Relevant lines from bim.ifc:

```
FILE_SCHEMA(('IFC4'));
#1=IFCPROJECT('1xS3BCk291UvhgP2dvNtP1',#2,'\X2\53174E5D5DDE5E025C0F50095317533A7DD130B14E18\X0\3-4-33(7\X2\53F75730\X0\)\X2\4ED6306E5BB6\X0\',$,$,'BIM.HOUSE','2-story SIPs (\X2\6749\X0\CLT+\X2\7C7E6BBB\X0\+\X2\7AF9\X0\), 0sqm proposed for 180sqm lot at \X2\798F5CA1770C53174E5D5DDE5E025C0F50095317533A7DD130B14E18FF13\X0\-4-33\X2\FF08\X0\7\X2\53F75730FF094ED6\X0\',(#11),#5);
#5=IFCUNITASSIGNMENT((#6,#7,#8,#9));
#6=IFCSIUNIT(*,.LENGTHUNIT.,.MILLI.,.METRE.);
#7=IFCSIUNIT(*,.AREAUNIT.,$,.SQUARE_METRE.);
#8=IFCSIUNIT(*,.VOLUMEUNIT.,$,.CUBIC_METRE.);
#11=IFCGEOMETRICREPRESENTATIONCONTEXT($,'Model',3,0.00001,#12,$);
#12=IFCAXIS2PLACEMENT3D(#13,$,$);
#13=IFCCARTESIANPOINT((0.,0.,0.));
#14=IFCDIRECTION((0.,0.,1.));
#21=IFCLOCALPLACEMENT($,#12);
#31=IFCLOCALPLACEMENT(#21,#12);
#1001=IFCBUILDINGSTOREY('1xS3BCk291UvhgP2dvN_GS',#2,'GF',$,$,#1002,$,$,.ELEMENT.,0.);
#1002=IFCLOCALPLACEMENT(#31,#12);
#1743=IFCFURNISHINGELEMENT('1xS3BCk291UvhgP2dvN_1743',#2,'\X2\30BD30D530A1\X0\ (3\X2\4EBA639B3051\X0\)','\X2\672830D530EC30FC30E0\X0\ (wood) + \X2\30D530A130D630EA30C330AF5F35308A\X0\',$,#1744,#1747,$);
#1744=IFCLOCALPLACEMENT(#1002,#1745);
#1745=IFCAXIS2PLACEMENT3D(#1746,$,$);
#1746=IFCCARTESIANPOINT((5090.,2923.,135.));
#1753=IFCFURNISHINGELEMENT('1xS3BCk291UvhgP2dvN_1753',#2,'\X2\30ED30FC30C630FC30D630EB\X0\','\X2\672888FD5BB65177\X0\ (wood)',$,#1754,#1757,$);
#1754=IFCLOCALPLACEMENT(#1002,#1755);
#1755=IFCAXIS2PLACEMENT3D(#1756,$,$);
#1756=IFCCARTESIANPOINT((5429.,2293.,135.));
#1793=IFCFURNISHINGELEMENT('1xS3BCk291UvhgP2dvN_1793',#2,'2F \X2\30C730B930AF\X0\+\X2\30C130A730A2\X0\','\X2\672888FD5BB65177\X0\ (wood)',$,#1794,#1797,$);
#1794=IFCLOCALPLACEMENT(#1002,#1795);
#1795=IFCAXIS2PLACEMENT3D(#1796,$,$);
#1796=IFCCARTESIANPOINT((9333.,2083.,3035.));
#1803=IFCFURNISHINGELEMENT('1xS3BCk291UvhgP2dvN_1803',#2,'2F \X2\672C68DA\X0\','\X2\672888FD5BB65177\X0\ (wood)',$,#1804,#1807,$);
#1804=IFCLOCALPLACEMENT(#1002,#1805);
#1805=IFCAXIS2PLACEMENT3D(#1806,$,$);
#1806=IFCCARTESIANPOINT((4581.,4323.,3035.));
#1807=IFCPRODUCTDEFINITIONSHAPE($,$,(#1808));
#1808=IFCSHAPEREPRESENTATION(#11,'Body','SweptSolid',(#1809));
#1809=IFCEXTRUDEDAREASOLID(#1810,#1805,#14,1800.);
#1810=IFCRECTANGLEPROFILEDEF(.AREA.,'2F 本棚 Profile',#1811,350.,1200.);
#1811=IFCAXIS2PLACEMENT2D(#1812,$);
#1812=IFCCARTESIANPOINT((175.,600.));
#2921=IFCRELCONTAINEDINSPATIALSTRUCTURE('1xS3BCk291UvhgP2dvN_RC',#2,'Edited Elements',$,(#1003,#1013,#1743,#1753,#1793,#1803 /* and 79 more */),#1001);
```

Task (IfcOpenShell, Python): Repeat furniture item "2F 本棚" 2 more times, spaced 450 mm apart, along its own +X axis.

```python
import ifcopenshell
import ifcopenshell.api.geometry
import ifcopenshell.api.root
import ifcopenshell.util.element
import ifcopenshell.util.placement

model = ifcopenshell.open("bim.ifc")


def reuse_history(source, copy):
    """copy_class also copies each property set's owner history, people and application; keep the originals."""
    for rel in copy.IsDefinedBy:
        if rel.is_a("IfcRelDefinesByProperties") and (history := rel.RelatingPropertyDefinition.OwnerHistory):
            rel.RelatingPropertyDefinition.OwnerHistory = source.OwnerHistory
            ifcopenshell.util.element.remove_deep2(model, history)


source = model.by_id(1803)
base = ifcopenshell.util.placement.get_local_placement(source.ObjectPlacement)
step = base[:3, 0] * 450.0

for i in range(1, 3):
    copy = ifcopenshell.api.root.copy_class(model, product=source)
    copy.Representation = ifcopenshell.util.element.copy_deep(
        model, source.Representation, exclude=["IfcGeometricRepresentationContext", "IfcRepresentationMap"]
    )
    reuse_history(source, copy)
    matrix = base.copy()
    matrix[:3, 3] += i * step
    print("added at", matrix[:3, 3].round(3) + 0.0)
    ifcopenshell.api.geometry.edit_object_placement(model, product=copy, matrix=matrix, is_si=False)

model.write("bim_v2.ifc")
```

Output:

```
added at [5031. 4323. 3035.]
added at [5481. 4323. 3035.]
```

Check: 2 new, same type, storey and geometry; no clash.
